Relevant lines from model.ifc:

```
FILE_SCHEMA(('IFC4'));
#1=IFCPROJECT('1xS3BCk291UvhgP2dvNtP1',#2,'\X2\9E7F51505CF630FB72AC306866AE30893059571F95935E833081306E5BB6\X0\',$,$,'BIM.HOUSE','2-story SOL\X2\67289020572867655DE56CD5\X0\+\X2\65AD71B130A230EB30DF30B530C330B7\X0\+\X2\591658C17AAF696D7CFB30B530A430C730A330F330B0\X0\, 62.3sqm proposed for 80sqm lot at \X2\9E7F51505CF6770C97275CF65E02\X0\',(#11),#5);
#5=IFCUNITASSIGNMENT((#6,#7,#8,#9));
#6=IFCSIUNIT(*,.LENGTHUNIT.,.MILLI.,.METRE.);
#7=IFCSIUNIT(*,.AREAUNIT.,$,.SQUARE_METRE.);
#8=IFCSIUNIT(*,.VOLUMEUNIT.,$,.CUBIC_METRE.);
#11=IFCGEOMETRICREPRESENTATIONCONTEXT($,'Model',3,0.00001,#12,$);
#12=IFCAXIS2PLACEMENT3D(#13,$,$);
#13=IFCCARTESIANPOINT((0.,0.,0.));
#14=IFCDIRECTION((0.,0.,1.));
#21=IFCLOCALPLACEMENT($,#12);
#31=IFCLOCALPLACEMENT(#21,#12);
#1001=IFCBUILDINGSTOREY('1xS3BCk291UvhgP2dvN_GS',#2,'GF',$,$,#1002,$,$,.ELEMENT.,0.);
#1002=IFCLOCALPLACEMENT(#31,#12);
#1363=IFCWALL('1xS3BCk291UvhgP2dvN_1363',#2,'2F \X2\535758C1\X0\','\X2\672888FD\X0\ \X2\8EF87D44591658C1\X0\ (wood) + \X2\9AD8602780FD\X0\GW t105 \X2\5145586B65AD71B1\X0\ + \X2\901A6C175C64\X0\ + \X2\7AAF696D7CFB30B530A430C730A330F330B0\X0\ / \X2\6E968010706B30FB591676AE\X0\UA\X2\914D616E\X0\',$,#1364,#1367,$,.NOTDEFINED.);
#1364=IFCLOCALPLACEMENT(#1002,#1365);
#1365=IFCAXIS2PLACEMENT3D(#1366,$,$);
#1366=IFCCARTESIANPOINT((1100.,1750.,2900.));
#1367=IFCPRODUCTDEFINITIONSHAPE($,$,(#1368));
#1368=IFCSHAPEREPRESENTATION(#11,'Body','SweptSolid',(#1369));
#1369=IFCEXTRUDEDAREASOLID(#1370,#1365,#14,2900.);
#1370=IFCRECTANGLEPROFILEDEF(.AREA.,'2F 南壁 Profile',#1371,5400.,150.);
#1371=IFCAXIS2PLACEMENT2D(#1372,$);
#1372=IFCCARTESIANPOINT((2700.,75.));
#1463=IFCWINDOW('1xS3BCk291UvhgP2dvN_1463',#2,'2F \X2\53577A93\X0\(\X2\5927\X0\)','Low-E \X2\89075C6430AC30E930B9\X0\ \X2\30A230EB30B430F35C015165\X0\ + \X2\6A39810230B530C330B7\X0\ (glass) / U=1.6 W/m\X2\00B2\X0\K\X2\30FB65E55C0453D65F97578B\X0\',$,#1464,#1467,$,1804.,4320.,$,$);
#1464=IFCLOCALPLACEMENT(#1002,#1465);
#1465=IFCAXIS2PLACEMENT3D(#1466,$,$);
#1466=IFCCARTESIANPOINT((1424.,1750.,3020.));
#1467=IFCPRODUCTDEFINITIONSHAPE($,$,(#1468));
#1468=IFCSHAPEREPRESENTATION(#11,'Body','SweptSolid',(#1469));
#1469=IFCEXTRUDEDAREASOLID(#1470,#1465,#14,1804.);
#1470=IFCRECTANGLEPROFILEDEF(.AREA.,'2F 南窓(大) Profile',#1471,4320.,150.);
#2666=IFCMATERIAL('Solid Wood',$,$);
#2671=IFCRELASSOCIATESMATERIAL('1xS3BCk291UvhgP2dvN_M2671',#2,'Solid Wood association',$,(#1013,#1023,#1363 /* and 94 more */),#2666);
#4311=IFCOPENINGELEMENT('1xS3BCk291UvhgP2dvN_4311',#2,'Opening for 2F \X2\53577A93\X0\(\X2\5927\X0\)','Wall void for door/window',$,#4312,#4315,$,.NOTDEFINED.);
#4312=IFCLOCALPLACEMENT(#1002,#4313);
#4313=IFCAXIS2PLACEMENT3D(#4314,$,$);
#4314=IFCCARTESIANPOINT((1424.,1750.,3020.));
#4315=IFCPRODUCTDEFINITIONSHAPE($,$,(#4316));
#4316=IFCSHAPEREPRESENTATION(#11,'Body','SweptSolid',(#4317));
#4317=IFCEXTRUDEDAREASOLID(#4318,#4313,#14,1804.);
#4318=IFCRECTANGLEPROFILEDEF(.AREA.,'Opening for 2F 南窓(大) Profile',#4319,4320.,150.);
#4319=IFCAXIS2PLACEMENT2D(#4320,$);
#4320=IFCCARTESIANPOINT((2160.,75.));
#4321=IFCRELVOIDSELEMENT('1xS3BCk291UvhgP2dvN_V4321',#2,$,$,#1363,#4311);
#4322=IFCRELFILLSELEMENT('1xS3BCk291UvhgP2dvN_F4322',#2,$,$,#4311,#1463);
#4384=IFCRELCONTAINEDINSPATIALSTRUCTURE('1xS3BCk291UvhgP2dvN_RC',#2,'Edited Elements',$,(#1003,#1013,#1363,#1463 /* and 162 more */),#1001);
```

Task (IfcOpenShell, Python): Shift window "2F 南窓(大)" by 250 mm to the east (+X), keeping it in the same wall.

```python
import ifcopenshell
import ifcopenshell.api.geometry
import ifcopenshell.util.placement

model = ifcopenshell.open("model.ifc")

window = model.by_guid("1xS3BCk291UvhgP2dvN_1463")
opening = window.FillsVoids[0].RelatingOpeningElement
wall = opening.VoidsElements[0].RelatingBuildingElement

wall_matrix = ifcopenshell.util.placement.get_local_placement(wall.ObjectPlacement)
shift = wall_matrix[:3, 0] * 250.0
before = ifcopenshell.util.placement.get_local_placement(window.ObjectPlacement)[:3, 3].copy()

# The window is not placed relative to its opening, so move both.
for product in (opening, window):
    matrix = ifcopenshell.util.placement.get_local_placement(product.ObjectPlacement)
    matrix[:3, 3] += shift
    ifcopenshell.api.geometry.edit_object_placement(model, product=product, matrix=matrix, is_si=False)

after = ifcopenshell.util.placement.get_local_placement(window.ObjectPlacement)[:3, 3]
print("window moved by", (after - before).round(3) + 0.0)

model.write("model_v2.ifc")
```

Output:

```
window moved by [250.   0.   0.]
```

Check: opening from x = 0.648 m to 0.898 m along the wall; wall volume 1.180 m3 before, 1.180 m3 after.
